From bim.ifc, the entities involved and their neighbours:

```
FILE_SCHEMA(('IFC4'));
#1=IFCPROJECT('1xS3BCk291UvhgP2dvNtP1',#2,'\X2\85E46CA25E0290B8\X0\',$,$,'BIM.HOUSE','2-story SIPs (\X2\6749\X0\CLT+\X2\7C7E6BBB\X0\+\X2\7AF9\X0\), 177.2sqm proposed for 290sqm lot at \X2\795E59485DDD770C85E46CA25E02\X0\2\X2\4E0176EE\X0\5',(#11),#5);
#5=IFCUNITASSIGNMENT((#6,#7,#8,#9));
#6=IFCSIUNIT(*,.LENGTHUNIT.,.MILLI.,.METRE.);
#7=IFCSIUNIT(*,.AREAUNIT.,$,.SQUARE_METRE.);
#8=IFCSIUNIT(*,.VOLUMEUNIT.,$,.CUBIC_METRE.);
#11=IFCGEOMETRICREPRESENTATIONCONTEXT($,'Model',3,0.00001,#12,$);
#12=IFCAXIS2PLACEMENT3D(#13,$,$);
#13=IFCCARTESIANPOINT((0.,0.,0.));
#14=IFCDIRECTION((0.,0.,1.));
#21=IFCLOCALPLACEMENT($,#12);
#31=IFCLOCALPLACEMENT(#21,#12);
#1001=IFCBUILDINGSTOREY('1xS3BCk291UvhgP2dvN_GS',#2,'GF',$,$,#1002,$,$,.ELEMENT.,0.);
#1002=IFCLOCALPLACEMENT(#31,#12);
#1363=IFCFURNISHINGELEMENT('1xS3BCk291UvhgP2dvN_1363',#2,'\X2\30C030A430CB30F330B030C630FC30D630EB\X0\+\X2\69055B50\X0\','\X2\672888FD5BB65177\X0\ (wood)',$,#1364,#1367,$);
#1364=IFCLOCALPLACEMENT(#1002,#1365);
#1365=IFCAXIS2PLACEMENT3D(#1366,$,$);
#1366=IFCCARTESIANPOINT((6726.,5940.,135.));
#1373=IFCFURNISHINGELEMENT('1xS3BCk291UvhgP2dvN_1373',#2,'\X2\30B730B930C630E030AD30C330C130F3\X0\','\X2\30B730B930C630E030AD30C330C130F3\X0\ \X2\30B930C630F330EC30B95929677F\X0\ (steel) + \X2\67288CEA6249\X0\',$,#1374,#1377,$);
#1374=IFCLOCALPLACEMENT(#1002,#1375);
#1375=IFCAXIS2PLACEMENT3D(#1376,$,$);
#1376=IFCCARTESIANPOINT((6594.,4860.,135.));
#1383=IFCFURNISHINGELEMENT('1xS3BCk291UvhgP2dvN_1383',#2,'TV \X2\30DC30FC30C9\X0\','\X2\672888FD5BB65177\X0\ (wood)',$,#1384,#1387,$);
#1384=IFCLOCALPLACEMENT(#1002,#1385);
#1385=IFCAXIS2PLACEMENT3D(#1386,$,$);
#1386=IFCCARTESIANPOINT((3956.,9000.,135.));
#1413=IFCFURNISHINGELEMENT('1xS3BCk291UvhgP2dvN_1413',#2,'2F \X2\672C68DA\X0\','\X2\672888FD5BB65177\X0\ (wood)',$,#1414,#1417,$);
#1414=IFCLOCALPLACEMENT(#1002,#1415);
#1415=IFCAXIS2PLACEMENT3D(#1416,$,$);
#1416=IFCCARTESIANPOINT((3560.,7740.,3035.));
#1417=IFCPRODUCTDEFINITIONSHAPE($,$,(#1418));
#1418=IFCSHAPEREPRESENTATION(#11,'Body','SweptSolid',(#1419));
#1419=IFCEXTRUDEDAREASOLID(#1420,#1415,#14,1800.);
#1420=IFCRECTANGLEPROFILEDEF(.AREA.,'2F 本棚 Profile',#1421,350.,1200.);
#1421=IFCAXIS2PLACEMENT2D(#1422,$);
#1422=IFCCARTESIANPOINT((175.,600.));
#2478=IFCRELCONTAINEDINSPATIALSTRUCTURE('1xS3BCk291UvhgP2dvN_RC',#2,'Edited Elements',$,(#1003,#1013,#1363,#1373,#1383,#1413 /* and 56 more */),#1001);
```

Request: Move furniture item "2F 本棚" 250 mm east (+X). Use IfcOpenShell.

```python
import ifcopenshell
import ifcopenshell.api.geometry
import ifcopenshell.util.placement
import ifcopenshell.util.unit

model = ifcopenshell.open("bim.ifc")
unit_scale = ifcopenshell.util.unit.calculate_unit_scale(model)

item = model.by_guid("1xS3BCk291UvhgP2dvN_1413")
matrix = ifcopenshell.util.placement.get_local_placement(item.ObjectPlacement)
matrix[0, 3] += 0.25 / unit_scale
ifcopenshell.api.geometry.edit_object_placement(model, product=item, matrix=matrix, is_si=False)

print(ifcopenshell.util.placement.get_local_placement(item.ObjectPlacement).round(3) + 0.0)

model.write("bim-out.ifc")
```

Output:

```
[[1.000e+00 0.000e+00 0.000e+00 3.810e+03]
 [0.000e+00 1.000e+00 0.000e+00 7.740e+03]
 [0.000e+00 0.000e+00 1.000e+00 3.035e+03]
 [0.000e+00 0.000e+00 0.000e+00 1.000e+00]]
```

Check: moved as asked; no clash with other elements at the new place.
